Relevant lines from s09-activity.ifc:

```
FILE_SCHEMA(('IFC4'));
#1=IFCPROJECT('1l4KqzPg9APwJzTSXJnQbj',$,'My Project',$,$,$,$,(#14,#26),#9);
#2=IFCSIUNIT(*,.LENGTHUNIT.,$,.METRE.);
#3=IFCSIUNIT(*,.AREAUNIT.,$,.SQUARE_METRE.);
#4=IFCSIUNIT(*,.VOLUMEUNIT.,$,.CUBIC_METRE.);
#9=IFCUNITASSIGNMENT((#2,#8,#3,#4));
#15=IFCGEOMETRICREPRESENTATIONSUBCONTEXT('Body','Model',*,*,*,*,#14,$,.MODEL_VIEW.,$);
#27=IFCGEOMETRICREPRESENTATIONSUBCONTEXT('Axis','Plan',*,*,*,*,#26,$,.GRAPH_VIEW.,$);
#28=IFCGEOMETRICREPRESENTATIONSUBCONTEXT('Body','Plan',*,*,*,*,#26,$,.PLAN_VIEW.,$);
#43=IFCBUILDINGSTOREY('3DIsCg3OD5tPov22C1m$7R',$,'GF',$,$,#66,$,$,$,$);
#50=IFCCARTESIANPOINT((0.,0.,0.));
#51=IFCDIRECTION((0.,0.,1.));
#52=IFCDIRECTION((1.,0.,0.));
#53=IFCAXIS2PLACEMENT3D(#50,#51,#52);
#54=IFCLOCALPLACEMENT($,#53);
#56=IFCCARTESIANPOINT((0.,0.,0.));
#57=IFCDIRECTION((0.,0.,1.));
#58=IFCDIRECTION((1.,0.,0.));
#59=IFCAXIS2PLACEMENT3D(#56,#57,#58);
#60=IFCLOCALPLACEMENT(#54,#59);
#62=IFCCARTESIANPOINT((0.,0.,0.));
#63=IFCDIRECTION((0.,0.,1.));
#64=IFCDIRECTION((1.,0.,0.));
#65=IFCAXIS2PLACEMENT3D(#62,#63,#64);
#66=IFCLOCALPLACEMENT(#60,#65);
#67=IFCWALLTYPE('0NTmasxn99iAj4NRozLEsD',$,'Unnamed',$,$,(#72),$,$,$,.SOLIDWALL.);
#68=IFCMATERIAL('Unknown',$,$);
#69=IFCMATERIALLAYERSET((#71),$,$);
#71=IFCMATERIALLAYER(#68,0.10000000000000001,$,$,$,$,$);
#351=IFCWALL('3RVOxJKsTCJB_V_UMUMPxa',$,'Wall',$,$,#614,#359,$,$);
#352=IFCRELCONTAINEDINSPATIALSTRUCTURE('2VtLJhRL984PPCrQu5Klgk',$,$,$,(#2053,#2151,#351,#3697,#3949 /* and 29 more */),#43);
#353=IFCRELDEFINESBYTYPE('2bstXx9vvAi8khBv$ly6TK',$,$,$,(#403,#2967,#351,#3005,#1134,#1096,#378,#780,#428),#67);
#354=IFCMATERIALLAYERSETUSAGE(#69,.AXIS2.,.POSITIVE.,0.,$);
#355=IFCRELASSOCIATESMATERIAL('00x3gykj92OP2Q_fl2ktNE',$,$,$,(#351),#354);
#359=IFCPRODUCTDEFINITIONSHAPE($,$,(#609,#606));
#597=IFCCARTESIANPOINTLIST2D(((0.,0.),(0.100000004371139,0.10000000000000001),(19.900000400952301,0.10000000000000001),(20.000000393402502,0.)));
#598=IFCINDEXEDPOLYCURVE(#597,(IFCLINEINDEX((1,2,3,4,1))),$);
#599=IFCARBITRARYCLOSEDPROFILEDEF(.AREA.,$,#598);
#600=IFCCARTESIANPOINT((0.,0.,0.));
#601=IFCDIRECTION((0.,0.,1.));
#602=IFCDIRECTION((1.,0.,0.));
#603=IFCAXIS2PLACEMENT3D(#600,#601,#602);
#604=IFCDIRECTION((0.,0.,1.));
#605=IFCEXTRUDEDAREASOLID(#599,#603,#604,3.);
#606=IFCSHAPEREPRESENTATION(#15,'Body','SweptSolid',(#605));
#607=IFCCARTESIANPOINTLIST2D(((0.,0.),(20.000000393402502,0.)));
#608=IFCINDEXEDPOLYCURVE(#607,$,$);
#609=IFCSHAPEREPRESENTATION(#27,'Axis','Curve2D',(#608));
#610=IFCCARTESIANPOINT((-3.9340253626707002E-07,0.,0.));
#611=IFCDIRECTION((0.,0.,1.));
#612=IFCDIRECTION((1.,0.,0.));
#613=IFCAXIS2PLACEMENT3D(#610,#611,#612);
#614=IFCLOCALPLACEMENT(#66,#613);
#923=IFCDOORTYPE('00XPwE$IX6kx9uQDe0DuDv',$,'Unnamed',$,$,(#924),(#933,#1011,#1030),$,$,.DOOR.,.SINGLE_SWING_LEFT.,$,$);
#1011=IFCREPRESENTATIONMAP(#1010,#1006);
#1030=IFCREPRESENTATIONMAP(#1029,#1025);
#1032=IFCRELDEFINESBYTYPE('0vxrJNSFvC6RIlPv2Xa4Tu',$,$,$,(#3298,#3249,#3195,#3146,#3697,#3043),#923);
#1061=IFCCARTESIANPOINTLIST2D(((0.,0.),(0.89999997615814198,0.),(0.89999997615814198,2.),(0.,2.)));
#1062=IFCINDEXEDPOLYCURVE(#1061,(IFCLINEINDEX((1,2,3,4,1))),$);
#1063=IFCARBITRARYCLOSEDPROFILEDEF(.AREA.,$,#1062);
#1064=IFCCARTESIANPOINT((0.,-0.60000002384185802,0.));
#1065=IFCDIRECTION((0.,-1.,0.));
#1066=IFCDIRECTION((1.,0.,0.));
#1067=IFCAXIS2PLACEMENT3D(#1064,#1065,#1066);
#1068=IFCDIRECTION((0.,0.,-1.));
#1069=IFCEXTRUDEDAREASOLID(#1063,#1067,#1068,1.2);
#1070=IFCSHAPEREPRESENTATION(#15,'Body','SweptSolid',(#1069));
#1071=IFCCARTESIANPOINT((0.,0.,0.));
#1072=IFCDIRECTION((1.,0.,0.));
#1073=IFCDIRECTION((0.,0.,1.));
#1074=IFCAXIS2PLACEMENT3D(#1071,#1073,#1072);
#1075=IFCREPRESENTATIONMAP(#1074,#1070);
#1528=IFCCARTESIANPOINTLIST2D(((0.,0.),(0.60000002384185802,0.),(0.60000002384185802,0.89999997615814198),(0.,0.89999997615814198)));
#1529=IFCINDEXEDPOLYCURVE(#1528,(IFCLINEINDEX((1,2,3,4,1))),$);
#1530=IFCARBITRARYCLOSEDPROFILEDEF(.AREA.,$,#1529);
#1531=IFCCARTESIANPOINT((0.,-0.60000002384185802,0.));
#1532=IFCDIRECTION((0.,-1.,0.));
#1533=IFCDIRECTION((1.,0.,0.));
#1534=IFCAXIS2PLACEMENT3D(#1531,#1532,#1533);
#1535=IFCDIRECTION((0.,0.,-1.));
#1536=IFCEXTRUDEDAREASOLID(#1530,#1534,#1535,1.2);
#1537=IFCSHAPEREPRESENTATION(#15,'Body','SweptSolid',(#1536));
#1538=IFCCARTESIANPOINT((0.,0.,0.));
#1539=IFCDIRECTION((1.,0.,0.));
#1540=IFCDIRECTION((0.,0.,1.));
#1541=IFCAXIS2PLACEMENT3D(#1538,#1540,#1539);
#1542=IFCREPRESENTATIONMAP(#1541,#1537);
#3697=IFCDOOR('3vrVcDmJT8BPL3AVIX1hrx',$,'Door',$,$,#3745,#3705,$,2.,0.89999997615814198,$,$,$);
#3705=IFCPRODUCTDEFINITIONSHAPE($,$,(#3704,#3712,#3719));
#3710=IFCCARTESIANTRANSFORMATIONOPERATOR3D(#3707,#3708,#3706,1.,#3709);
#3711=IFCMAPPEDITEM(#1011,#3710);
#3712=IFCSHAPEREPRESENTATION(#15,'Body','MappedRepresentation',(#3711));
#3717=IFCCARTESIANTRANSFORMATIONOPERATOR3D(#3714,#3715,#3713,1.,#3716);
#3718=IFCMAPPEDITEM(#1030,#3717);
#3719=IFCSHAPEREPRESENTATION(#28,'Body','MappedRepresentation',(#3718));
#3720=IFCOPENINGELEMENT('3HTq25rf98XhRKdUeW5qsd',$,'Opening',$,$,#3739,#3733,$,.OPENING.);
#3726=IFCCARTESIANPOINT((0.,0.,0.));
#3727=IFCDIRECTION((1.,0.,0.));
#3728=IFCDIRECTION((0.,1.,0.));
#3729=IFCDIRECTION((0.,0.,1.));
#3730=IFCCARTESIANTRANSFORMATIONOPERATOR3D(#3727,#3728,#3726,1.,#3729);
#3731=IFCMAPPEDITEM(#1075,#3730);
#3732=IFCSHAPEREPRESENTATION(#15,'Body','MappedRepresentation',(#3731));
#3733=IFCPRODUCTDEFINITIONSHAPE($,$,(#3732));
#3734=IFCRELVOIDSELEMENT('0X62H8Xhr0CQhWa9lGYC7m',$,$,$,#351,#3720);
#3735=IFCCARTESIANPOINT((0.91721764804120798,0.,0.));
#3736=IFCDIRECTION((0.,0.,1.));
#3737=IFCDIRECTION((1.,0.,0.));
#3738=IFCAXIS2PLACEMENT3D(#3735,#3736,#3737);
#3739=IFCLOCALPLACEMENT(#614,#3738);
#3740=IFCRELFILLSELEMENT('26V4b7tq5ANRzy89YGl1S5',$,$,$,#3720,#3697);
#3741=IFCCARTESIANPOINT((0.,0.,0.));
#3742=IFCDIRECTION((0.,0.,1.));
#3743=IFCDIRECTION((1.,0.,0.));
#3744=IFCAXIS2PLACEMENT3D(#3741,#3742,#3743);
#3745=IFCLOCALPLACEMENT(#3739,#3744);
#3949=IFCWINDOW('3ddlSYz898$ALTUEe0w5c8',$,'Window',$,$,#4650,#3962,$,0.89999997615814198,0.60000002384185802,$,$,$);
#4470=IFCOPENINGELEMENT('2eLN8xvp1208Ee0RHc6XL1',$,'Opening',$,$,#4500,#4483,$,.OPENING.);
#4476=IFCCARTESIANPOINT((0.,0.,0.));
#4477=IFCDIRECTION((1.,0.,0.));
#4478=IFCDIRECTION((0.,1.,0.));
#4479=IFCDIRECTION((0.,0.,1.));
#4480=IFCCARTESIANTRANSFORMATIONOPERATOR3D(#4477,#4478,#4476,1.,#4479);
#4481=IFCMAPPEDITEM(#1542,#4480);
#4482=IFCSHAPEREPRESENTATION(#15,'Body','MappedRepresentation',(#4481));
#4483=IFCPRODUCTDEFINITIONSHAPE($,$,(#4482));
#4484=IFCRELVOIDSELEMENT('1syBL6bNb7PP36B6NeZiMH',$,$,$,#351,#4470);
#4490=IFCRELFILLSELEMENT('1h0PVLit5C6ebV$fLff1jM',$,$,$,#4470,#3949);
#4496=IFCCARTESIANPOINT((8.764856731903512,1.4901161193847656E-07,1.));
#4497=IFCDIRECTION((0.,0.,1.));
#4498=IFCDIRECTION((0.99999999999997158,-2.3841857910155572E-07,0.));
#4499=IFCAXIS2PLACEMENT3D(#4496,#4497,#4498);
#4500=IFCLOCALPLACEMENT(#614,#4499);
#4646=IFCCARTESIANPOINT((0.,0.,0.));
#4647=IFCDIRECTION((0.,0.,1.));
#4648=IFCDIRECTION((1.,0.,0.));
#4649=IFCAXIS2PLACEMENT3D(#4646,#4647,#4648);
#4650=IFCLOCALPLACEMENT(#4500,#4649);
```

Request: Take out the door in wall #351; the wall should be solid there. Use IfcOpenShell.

```python
import ifcopenshell
import ifcopenshell.api.feature
import ifcopenshell.api.root
import ifcopenshell.geom
import ifcopenshell.util.shape

model = ifcopenshell.open("s09-activity.ifc")
settings = ifcopenshell.geom.settings()


def volume(element):
    """Net volume in cubic metres, openings subtracted."""
    shape = ifcopenshell.geom.create_shape(settings, element)
    return ifcopenshell.util.shape.get_volume(shape.geometry)


door = model.by_id(3697)
opening = door.FillsVoids[0].RelatingOpeningElement
wall = opening.VoidsElements[0].RelatingBuildingElement
before = volume(wall)

ifcopenshell.api.root.remove_product(model, product=door)
ifcopenshell.api.feature.remove_feature(model, feature=opening)

after = volume(wall)

print(f"wall volume {before:.3f} -> {after:.3f} m3")

model.write("s09-activity_updated.ifc")
```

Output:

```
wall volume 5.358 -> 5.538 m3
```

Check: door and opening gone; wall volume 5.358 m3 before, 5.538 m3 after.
